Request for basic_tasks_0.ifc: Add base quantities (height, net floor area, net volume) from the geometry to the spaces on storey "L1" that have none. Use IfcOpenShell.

First a look at what the model holds.

```python
import ifcopenshell
import ifcopenshell.util.element
import ifcopenshell.util.unit

model = ifcopenshell.open("basic_tasks_0.ifc")
print(model.schema)
for unit_type in ("LENGTHUNIT", "AREAUNIT", "VOLUMEUNIT"):
    print(unit_type, ifcopenshell.util.unit.calculate_unit_scale(model, unit_type))
storey = next(s for s in model.by_type("IfcBuildingStorey") if s.Name == "L1")
spaces = [e for e in ifcopenshell.util.element.get_decomposition(storey) if e.is_a("IfcSpace")]
for e in sorted(spaces, key=lambda e: e.id()):
    print(e.id(), e.is_a(), e.Name, list(ifcopenshell.util.element.get_psets(e, qtos_only=True)), sep=" | ")
```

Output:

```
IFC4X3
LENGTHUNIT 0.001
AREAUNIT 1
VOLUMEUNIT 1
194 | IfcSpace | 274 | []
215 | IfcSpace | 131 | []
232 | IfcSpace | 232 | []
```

```python
import ifcopenshell
import ifcopenshell.api.pset
import ifcopenshell.geom
import ifcopenshell.util.element
import ifcopenshell.util.shape
import ifcopenshell.util.unit

model = ifcopenshell.open("basic_tasks_0.ifc")
unit_scale = ifcopenshell.util.unit.calculate_unit_scale(model)
area_scale = ifcopenshell.util.unit.calculate_unit_scale(model, "AREAUNIT")
volume_scale = ifcopenshell.util.unit.calculate_unit_scale(model, "VOLUMEUNIT")
settings = ifcopenshell.geom.settings()

storey = next(s for s in model.by_type("IfcBuildingStorey") if s.Name == "L1")
spaces = [e for e in ifcopenshell.util.element.get_decomposition(storey) if e.is_a("IfcSpace")]

for e in sorted(spaces, key=lambda e: e.id()):
    if ifcopenshell.util.element.get_psets(e, qtos_only=True, should_inherit=False):
        continue
    # Geometry comes back in metres, in the element's own axes.
    shape = ifcopenshell.geom.create_shape(settings, e)
    values = {
        "Height": ifcopenshell.util.shape.get_z(shape.geometry) / unit_scale,
        "NetFloorArea": ifcopenshell.util.shape.get_footprint_area(shape.geometry) / area_scale,
        "NetVolume": ifcopenshell.util.shape.get_volume(shape.geometry) / volume_scale,
    }
    qto = ifcopenshell.api.pset.add_qto(model, product=e, name="Qto_SpaceBaseQuantities")
    ifcopenshell.api.pset.edit_qto(model, qto=qto, properties=values)
    print(e.id(), {k: round(v, 3) for k, v in values.items()})

model.write("basic_tasks_0_edited.ifc")
```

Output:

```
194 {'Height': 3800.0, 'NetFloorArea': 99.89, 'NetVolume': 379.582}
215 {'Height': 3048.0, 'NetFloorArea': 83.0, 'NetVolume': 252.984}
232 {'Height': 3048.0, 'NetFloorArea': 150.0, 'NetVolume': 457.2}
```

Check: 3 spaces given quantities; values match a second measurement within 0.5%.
